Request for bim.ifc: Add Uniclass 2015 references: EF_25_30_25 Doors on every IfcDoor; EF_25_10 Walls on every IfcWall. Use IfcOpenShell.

First a look at what the model holds.

```python
import ifcopenshell

model = ifcopenshell.open("bim.ifc")
print(model.schema)
print("classifications:", [c.Name for c in model.by_type("IfcClassification")])
for ifc_class in ("IfcDoor", "IfcRoof", "IfcStair", "IfcWall", "IfcWindow"):
    print(ifc_class, len(model.by_type(ifc_class)))
```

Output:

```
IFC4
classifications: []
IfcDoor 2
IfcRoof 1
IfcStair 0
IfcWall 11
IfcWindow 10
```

```python
import ifcopenshell
import ifcopenshell.api.classification

model = ifcopenshell.open("bim.ifc")

system = ifcopenshell.api.classification.add_classification(model, classification="Uniclass 2015")

codes = {
    "IfcDoor": ("EF_25_30_25", "Doors"),
    "IfcWall": ("EF_25_10", "Walls"),
}
for ifc_class, (code, name) in codes.items():
    products = model.by_type(ifc_class)
    ifcopenshell.api.classification.add_reference(
        model, products=products, classification=system, identification=code, name=name
    )
    print(code, len(products))

model.write("bim_rev.ifc")
```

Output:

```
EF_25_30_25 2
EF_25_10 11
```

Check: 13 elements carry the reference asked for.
